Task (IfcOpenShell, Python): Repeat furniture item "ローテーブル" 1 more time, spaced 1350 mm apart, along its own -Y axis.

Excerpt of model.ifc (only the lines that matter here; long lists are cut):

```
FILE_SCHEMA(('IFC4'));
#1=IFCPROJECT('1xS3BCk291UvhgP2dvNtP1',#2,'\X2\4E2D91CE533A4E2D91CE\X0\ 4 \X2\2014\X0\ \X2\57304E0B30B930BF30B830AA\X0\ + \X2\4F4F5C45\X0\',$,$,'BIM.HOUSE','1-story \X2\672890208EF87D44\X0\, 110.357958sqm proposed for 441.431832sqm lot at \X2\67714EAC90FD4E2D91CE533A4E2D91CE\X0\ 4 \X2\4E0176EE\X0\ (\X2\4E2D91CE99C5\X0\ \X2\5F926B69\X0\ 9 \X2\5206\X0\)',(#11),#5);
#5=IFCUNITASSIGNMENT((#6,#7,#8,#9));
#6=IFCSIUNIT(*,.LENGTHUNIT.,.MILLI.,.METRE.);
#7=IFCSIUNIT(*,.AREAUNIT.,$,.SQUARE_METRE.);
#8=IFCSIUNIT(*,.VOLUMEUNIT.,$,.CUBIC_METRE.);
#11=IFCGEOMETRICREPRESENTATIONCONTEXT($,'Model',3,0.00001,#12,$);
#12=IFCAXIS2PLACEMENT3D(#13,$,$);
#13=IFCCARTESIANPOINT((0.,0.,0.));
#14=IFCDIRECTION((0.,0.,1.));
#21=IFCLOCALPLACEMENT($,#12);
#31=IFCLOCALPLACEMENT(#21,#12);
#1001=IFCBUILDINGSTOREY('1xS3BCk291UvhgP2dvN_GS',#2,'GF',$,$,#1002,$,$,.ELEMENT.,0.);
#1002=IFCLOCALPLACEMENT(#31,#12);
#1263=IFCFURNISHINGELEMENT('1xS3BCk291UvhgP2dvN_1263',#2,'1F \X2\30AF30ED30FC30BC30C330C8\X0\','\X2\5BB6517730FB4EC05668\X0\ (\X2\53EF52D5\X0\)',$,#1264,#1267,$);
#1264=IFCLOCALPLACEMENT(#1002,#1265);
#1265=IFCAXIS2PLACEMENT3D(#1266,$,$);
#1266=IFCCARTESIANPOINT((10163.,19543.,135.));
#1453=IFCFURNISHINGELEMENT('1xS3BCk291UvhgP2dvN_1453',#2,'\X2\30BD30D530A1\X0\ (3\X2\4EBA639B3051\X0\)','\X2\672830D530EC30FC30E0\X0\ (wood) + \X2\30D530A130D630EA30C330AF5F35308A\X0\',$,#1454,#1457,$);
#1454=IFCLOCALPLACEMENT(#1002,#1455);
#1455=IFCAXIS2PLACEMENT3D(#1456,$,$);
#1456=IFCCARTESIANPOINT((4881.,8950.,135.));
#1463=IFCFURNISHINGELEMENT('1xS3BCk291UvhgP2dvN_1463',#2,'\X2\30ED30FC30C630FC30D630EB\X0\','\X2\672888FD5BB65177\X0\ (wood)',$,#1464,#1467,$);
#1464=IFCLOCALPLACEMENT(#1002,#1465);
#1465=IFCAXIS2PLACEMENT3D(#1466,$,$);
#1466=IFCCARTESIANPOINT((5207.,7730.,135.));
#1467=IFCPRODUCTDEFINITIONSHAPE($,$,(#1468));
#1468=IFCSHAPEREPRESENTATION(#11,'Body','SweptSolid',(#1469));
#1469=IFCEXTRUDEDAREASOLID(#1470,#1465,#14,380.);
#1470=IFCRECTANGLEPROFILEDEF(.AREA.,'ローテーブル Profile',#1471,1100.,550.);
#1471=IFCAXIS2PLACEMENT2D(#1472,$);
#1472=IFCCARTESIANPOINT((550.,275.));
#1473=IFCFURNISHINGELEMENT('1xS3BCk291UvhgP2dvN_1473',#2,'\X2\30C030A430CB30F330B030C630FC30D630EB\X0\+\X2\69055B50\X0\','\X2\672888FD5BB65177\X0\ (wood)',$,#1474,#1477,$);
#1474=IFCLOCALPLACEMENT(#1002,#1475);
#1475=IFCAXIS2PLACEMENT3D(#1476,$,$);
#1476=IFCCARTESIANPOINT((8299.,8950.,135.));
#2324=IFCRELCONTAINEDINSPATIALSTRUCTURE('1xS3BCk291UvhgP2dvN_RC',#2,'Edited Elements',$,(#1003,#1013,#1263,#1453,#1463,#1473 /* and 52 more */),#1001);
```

```python
import ifcopenshell
import ifcopenshell.api.geometry
import ifcopenshell.api.root
import ifcopenshell.util.element
import ifcopenshell.util.placement
import ifcopenshell.util.unit

model = ifcopenshell.open("model.ifc")
unit_scale = ifcopenshell.util.unit.calculate_unit_scale(model)


def reuse_history(source, copy):
    """copy_class also copies each property set's owner history, people and application; keep the originals."""
    for rel in copy.IsDefinedBy:
        if rel.is_a("IfcRelDefinesByProperties") and (history := rel.RelatingPropertyDefinition.OwnerHistory):
            rel.RelatingPropertyDefinition.OwnerHistory = source.OwnerHistory
            ifcopenshell.util.element.remove_deep2(model, history)


source = model.by_id(1463)
base = ifcopenshell.util.placement.get_local_placement(source.ObjectPlacement)
step = -base[:3, 1] * 1.35 / unit_scale

for i in range(1, 2):
    copy = ifcopenshell.api.root.copy_class(model, product=source)
    copy.Representation = ifcopenshell.util.element.copy_deep(
        model, source.Representation, exclude=["IfcGeometricRepresentationContext", "IfcRepresentationMap"]
    )
    reuse_history(source, copy)
    matrix = base.copy()
    matrix[:3, 3] += i * step
    print("added at", matrix[:3, 3].round(3) + 0.0)
    ifcopenshell.api.geometry.edit_object_placement(model, product=copy, matrix=matrix, is_si=False)

model.write("model_edited.ifc")
```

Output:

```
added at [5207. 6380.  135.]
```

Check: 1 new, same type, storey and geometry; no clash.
